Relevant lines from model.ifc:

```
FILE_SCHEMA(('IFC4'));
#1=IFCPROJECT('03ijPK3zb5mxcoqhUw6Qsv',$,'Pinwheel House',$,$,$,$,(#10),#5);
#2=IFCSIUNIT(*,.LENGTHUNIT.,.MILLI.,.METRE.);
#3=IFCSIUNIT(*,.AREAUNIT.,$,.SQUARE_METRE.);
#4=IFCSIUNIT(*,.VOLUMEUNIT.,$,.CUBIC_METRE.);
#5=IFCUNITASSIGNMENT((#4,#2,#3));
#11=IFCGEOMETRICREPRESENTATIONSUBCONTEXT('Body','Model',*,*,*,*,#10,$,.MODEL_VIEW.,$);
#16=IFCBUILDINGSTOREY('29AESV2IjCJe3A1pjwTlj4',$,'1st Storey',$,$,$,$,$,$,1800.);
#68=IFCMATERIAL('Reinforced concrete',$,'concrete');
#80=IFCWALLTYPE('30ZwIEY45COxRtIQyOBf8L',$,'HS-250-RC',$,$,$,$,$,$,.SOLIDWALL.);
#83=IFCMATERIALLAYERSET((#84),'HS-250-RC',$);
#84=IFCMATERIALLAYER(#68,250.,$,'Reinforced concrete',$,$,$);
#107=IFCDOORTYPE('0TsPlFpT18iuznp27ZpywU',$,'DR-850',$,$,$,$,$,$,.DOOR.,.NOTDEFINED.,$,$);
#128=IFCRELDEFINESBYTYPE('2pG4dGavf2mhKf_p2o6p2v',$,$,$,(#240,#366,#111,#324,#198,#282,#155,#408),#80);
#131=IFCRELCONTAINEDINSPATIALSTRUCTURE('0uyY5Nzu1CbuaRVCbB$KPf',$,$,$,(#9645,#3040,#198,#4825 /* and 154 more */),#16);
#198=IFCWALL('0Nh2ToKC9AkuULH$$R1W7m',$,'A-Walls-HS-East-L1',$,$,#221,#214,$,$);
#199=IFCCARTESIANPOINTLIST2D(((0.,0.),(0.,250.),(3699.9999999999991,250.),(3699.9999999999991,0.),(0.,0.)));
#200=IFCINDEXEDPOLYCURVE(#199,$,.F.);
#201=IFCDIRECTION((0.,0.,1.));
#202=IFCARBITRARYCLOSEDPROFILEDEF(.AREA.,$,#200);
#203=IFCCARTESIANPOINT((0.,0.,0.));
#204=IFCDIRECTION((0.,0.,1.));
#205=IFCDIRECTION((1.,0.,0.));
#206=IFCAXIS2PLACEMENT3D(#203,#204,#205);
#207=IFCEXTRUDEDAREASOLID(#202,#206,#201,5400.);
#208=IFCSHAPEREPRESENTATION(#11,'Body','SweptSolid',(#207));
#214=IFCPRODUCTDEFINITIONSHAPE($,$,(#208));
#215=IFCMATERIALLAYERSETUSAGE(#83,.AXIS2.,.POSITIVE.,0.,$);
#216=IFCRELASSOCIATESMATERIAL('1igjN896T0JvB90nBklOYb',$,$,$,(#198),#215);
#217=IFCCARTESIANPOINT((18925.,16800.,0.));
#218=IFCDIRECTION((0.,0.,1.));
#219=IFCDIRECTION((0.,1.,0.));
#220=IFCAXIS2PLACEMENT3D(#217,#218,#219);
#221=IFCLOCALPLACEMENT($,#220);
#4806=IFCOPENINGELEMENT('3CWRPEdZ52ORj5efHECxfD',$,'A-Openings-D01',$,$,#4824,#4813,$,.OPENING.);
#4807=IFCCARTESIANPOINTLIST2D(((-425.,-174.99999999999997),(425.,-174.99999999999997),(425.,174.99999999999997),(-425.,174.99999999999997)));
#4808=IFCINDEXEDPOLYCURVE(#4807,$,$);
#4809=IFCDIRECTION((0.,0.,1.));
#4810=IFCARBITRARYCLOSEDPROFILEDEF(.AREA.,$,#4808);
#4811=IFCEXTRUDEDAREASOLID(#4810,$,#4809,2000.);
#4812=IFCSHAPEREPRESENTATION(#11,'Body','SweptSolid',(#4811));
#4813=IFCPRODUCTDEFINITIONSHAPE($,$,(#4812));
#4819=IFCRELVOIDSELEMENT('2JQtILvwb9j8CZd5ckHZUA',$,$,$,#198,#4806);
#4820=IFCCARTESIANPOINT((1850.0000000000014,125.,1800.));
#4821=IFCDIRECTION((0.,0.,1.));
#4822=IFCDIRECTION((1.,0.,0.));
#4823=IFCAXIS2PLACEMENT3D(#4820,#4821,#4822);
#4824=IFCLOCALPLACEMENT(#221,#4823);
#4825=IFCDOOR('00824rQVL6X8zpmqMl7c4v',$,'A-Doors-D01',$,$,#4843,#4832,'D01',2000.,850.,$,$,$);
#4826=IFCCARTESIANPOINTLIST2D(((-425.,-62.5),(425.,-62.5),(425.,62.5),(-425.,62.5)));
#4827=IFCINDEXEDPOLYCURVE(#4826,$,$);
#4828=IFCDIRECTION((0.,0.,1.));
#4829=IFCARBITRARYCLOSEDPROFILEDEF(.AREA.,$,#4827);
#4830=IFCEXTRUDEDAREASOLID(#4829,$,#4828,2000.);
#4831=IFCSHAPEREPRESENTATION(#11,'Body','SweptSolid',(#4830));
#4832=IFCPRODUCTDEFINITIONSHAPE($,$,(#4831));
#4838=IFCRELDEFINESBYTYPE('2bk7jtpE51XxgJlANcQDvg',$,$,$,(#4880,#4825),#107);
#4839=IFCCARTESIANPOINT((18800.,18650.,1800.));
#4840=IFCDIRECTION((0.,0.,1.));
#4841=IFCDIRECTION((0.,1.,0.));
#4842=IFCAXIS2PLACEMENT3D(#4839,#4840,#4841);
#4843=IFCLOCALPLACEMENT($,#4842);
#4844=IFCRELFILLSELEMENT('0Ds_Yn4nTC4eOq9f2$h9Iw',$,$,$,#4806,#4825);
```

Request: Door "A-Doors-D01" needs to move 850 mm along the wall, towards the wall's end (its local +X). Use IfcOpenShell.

```python
import ifcopenshell
import ifcopenshell.api.geometry
import ifcopenshell.util.placement
import ifcopenshell.util.unit

model = ifcopenshell.open("model.ifc")
unit_scale = ifcopenshell.util.unit.calculate_unit_scale(model)

door = model.by_guid("00824rQVL6X8zpmqMl7c4v")
opening = door.FillsVoids[0].RelatingOpeningElement
wall = opening.VoidsElements[0].RelatingBuildingElement

wall_matrix = ifcopenshell.util.placement.get_local_placement(wall.ObjectPlacement)
shift = wall_matrix[:3, 0] * 0.85 / unit_scale
before = ifcopenshell.util.placement.get_local_placement(door.ObjectPlacement)[:3, 3].copy()

# The door is not placed relative to its opening, so move both.
for product in (opening, door):
    matrix = ifcopenshell.util.placement.get_local_placement(product.ObjectPlacement)
    matrix[:3, 3] += shift
    ifcopenshell.api.geometry.edit_object_placement(model, product=product, matrix=matrix, is_si=False)

after = ifcopenshell.util.placement.get_local_placement(door.ObjectPlacement)[:3, 3]
print("door moved by", (after - before).round(3) + 0.0)

model.write("model_v2.ifc")
```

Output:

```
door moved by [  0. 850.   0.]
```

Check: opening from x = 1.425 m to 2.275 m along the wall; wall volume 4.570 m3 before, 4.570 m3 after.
